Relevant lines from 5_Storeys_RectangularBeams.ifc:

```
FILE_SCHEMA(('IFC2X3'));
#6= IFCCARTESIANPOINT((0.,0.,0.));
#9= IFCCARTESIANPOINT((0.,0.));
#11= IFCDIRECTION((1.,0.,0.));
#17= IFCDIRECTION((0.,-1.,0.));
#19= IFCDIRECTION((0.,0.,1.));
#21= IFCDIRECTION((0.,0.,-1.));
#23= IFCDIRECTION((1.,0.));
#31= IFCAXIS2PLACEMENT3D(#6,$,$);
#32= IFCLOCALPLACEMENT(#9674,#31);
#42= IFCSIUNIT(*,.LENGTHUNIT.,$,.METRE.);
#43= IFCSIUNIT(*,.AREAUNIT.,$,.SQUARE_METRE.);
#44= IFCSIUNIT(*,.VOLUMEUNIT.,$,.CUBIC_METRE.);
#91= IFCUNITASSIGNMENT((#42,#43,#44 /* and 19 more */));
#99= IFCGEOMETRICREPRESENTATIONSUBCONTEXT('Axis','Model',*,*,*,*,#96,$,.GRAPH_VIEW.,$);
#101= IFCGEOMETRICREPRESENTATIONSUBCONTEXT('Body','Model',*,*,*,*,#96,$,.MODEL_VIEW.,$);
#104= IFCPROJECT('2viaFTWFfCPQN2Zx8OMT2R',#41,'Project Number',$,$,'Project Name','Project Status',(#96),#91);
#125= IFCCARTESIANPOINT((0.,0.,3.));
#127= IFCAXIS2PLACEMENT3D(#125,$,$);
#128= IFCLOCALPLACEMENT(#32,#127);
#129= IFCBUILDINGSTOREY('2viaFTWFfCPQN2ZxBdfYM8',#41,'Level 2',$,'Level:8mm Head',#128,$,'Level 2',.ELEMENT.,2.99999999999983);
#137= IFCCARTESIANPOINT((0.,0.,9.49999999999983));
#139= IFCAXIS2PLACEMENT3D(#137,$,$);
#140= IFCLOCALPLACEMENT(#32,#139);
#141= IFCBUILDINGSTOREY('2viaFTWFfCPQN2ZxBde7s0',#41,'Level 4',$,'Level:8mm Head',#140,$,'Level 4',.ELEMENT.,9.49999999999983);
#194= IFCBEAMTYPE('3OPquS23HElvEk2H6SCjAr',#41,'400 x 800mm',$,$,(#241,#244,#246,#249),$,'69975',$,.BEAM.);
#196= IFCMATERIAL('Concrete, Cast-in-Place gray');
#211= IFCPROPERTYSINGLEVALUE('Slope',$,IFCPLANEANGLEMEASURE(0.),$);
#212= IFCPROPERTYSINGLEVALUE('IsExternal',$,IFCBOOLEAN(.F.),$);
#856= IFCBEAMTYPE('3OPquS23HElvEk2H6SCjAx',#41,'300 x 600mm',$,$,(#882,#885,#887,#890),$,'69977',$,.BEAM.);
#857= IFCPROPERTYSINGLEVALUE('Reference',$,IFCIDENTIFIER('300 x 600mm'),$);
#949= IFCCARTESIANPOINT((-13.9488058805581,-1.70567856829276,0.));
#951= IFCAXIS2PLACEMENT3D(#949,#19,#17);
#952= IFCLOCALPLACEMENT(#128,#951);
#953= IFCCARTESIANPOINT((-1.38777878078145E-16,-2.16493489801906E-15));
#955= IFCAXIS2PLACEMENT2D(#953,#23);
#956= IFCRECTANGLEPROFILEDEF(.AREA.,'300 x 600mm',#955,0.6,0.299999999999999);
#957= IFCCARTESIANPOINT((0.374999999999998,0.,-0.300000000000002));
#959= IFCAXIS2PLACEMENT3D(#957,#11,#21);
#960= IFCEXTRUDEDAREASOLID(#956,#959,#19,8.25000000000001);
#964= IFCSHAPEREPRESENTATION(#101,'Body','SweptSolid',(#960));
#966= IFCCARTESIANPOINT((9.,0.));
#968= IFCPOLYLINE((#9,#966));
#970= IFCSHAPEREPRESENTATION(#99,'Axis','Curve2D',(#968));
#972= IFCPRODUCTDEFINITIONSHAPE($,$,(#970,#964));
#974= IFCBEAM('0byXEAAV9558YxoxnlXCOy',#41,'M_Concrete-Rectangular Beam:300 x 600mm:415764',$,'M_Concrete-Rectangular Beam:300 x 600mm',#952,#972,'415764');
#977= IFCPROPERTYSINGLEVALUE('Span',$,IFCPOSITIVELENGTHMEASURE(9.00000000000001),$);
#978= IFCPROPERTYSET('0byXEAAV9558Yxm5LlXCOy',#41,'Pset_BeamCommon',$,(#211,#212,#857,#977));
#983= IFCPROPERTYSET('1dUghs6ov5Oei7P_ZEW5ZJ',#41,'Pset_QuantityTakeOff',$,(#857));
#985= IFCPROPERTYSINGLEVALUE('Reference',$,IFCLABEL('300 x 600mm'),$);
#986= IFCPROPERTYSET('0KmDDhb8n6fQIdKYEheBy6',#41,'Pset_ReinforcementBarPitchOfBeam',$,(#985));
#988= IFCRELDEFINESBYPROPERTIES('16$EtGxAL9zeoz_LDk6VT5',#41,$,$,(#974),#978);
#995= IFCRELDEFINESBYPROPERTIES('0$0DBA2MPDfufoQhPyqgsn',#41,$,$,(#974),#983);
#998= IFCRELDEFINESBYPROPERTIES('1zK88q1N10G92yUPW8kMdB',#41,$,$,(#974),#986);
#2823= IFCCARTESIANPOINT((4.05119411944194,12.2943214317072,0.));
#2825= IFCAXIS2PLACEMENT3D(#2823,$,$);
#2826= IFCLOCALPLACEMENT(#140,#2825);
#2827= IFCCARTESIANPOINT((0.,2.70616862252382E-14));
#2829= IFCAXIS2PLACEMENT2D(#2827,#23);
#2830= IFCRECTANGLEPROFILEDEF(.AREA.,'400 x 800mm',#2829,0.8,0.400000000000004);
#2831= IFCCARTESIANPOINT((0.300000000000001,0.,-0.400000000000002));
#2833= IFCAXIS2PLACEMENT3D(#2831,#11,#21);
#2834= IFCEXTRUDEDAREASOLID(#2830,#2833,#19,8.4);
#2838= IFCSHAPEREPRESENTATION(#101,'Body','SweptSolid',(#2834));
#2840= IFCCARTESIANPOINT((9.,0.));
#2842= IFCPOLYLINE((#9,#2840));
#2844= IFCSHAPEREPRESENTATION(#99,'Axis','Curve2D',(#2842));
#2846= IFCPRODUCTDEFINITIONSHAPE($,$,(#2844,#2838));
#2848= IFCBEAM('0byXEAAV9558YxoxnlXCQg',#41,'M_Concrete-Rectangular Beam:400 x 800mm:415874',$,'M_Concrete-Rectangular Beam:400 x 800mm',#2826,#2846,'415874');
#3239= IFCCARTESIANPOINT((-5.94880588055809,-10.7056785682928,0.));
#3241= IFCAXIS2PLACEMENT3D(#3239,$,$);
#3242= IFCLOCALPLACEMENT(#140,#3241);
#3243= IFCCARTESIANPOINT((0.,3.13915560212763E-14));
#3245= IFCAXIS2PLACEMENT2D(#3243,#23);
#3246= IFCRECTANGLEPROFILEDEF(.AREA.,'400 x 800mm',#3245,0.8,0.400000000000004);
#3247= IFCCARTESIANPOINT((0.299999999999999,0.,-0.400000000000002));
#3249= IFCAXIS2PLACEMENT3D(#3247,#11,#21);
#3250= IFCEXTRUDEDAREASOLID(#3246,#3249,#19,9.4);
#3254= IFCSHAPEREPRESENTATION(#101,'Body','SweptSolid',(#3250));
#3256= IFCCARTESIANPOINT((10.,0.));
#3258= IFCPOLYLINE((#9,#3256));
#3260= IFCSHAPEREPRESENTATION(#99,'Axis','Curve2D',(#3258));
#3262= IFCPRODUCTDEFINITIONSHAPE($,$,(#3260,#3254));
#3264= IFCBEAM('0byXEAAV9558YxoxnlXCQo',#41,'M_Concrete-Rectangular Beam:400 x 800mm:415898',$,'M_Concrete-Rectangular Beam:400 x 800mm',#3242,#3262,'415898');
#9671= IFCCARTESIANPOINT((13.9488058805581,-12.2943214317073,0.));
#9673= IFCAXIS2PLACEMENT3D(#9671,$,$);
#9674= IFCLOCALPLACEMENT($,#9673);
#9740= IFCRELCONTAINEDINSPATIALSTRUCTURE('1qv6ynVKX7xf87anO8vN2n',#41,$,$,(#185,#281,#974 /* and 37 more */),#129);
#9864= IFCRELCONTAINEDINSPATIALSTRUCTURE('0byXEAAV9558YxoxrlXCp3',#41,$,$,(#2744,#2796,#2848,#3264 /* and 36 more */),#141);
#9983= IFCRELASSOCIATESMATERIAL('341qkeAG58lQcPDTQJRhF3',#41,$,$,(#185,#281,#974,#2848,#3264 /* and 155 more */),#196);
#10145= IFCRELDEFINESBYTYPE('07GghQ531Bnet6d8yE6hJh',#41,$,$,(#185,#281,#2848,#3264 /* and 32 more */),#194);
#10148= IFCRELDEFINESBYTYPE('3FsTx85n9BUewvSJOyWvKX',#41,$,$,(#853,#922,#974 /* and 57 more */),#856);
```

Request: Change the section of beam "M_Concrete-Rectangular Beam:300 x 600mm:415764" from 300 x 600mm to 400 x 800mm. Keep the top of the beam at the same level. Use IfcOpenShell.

```python
import ifcopenshell
import ifcopenshell.api.pset
import ifcopenshell.api.type
import ifcopenshell.util.element
import ifcopenshell.util.representation

model = ifcopenshell.open("5_Storeys_RectangularBeams.ifc")

member = model.by_guid("0byXEAAV9558YxoxnlXCOy")
source = next(p for p in model.by_type("IfcRectangleProfileDef") if p.ProfileName == "400 x 800mm")

body = ifcopenshell.util.representation.get_representation(member, "Model", "Body")
solid = body.Items[0]
old_profile = solid.SweptArea

# Copy the section's sizes but keep this member's own profile position.
profile = ifcopenshell.util.element.copy(model, source)
# Profiles are centred, so shift by half the change in depth to hold the top.
shift = (old_profile.XDim - profile.XDim) / 2
x, y = old_profile.Position.Location.Coordinates
up = (-1.0, 0.0)  # upwards, in the solid's own plane
location = model.createIfcCartesianPoint((x + up[0] * shift, y + up[1] * shift))
profile.Position = model.createIfcAxis2Placement2D(location, old_profile.Position.RefDirection)
solid.SweptArea = profile
if not model.get_total_inverses(old_profile):
    ifcopenshell.util.element.remove_deep2(model, old_profile)

new_type = model.by_guid("3OPquS23HElvEk2H6SCjAr")
ifcopenshell.api.type.assign_type(
    model, related_objects=[member], relating_type=new_type, should_map_representations=False
)
member.Name = member.Name.replace("300 x 600mm", "400 x 800mm")
member.ObjectType = "M_Concrete-Rectangular Beam:400 x 800mm"
pset = model.by_id(ifcopenshell.util.element.get_pset(member, "Pset_BeamCommon", should_inherit=False)["id"])
ifcopenshell.api.pset.edit_pset(model, pset=pset, properties={"Reference": "400 x 800mm"})
pset = model.by_id(ifcopenshell.util.element.get_pset(member, "Pset_QuantityTakeOff", should_inherit=False)["id"])
ifcopenshell.api.pset.edit_pset(model, pset=pset, properties={"Reference": "400 x 800mm"})
pset = model.by_id(ifcopenshell.util.element.get_pset(member, "Pset_ReinforcementBarPitchOfBeam", should_inherit=False)["id"])
ifcopenshell.api.pset.edit_pset(model, pset=pset, properties={"Reference": "400 x 800mm"})

print(solid.SweptArea)

model.write("5_Storeys_RectangularBeams_updated.ifc")
```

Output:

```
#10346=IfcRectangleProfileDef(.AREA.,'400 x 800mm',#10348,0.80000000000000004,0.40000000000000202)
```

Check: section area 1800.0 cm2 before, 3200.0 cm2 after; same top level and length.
